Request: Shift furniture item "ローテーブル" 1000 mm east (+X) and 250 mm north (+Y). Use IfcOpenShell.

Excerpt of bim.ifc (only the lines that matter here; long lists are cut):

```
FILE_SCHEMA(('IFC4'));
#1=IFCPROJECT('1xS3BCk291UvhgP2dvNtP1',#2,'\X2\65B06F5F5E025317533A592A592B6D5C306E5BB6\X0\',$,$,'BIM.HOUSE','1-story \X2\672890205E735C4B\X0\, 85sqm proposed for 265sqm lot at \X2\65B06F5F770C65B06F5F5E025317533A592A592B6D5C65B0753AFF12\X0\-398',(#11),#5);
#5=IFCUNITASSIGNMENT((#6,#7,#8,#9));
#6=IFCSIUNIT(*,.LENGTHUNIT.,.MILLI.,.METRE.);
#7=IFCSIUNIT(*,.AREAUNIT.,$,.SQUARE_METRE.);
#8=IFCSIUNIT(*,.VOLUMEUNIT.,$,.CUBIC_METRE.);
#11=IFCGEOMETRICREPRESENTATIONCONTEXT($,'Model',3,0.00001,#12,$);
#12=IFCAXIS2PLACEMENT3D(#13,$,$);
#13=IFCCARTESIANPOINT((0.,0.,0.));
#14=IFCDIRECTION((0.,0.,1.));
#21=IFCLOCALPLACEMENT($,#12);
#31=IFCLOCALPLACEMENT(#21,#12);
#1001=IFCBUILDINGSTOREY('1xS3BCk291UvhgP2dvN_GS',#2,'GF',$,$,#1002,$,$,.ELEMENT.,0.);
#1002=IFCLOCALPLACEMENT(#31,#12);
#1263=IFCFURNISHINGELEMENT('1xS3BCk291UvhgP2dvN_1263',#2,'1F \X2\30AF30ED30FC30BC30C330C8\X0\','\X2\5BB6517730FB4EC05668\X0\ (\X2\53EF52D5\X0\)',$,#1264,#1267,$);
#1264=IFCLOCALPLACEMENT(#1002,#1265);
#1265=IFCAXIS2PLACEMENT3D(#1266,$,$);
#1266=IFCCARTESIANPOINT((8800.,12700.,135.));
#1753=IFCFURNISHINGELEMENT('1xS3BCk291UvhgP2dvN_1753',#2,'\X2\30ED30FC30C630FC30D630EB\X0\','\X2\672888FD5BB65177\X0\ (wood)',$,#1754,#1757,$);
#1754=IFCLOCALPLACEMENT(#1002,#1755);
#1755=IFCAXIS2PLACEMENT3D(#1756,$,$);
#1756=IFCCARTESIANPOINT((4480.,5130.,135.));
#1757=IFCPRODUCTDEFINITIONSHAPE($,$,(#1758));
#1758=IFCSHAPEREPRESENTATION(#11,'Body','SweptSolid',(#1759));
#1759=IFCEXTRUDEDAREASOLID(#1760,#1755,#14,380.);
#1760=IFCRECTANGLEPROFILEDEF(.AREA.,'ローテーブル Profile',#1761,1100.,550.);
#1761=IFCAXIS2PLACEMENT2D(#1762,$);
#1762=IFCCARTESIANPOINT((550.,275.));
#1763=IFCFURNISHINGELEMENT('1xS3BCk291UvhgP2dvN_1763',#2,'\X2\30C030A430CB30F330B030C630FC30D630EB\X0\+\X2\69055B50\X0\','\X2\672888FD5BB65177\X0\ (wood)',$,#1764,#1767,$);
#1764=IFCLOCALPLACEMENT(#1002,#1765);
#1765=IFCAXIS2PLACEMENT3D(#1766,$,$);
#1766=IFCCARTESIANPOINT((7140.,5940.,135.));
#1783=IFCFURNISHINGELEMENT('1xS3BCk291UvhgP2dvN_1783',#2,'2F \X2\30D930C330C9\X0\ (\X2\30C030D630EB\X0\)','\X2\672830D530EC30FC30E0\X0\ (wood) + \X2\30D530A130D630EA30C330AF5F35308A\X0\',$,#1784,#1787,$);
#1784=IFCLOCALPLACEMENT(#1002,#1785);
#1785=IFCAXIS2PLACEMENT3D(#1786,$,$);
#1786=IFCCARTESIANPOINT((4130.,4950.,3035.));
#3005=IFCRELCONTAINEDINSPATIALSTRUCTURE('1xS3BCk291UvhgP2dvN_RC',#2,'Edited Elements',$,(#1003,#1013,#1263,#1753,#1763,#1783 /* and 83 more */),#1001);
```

```python
import ifcopenshell
import ifcopenshell.api.geometry
import ifcopenshell.util.placement

model = ifcopenshell.open("bim.ifc")

item = model.by_id(1753)
matrix = ifcopenshell.util.placement.get_local_placement(item.ObjectPlacement)
matrix[0, 3] += 1000.0
matrix[1, 3] += 250.0
ifcopenshell.api.geometry.edit_object_placement(model, product=item, matrix=matrix, is_si=False)

print(ifcopenshell.util.placement.get_local_placement(item.ObjectPlacement).round(3) + 0.0)

model.write("bim-out.ifc")
```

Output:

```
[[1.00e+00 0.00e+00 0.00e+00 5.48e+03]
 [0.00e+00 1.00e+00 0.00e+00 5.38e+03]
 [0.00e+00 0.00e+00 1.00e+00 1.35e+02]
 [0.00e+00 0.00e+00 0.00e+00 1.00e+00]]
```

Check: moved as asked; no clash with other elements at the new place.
